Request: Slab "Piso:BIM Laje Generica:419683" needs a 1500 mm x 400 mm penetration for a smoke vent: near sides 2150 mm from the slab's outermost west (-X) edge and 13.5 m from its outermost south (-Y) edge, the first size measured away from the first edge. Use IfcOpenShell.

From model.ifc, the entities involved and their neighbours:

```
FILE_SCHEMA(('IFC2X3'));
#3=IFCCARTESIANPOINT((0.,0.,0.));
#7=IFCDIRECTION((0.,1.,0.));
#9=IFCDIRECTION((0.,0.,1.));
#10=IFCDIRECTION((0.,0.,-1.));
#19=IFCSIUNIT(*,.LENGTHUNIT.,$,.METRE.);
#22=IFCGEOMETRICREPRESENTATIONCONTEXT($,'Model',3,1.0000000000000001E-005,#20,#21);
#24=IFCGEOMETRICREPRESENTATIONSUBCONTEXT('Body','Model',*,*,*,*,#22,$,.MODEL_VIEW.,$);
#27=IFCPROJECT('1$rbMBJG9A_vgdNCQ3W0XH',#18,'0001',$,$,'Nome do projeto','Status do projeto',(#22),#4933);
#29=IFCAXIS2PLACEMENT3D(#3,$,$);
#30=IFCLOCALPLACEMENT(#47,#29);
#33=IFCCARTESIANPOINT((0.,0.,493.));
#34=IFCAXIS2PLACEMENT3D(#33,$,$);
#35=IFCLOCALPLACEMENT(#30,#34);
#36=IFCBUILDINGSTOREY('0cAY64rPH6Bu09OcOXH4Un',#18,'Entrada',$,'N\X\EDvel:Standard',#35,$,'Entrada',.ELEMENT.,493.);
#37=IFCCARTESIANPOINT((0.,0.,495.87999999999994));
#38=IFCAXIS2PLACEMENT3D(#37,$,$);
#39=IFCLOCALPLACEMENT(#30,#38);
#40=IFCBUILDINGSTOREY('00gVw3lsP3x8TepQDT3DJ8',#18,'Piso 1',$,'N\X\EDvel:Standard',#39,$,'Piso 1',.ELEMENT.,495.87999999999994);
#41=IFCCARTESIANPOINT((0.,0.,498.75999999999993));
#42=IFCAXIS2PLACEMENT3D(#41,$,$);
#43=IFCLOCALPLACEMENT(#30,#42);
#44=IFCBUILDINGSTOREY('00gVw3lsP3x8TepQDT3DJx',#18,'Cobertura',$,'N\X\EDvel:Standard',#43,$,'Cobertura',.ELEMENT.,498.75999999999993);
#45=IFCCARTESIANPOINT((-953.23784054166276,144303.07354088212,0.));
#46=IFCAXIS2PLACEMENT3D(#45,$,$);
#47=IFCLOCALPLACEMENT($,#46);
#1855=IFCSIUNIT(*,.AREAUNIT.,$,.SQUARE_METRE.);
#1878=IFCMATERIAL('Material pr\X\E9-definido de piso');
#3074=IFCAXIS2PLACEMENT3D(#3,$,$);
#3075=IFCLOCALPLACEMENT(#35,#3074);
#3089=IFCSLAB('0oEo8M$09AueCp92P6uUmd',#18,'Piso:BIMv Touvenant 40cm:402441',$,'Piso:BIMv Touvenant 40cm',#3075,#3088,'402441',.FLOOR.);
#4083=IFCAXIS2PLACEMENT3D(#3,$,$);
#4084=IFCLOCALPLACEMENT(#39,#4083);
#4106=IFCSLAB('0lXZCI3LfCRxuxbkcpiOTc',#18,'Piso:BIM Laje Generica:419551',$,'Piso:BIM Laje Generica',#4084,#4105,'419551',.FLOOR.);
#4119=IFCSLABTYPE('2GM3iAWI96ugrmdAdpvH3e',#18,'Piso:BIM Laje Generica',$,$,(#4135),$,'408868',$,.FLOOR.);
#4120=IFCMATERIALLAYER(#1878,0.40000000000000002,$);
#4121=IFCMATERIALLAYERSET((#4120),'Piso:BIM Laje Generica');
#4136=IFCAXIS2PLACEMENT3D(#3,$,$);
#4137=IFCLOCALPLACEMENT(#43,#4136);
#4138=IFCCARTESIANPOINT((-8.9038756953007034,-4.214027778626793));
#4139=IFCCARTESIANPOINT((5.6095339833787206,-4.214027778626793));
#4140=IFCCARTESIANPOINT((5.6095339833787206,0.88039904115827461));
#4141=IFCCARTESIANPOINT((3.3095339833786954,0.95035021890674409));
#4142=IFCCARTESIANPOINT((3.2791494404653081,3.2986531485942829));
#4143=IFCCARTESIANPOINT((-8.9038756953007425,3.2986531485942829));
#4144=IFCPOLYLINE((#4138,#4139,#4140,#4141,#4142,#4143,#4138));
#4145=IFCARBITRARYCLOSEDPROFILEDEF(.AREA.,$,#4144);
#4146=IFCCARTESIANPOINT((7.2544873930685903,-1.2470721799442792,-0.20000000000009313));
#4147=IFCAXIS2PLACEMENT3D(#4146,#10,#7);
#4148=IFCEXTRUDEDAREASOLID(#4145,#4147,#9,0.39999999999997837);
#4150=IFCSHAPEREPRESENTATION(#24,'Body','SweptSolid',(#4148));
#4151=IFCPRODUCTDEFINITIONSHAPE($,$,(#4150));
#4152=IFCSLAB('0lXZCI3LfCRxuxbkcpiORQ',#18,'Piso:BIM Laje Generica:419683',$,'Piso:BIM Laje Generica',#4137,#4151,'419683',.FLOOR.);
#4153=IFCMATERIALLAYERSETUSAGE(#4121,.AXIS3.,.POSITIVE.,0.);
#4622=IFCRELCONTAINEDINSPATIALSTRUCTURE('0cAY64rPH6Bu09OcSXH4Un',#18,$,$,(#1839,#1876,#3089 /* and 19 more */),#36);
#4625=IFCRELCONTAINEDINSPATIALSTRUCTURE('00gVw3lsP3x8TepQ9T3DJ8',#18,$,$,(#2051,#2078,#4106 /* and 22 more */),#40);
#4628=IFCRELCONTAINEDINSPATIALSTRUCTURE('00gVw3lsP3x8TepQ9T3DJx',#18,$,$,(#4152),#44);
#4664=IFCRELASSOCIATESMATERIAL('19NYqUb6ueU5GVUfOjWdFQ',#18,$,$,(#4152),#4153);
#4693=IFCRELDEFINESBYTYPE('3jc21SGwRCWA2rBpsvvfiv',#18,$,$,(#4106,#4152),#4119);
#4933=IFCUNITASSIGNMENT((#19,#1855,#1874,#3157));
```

```python
import numpy as np
import ifcopenshell
import ifcopenshell.api.feature
import ifcopenshell.api.geometry
import ifcopenshell.api.root
import ifcopenshell.geom
import ifcopenshell.util.placement
import ifcopenshell.util.representation
import ifcopenshell.util.shape
import ifcopenshell.util.unit

model = ifcopenshell.open("model.ifc")
unit_scale = ifcopenshell.util.unit.calculate_unit_scale(model)
settings = ifcopenshell.geom.settings()


def volume(element):
    """Net volume in cubic metres, openings subtracted."""
    shape = ifcopenshell.geom.create_shape(settings, element)
    return ifcopenshell.util.shape.get_volume(shape.geometry)


slab = model.by_id(4152)
before = volume(slab)

# Extent in the slab's own axes, in metres. The edges named are its -X and -Y sides.
slab_shape = ifcopenshell.geom.create_shape(settings, slab)
vertices = ifcopenshell.util.shape.get_vertices(slab_shape.geometry)
x_min, y_min, bottom = vertices.min(axis=0)
top = vertices[:, 2].max()

opening = ifcopenshell.api.root.create_entity(model, ifc_class="IfcOpeningElement", name="Smoke vent opening")
context = ifcopenshell.util.representation.get_context(model, "Model", "Body", "MODEL_VIEW")
width, depth = 1.5, 0.4
outline = [(0.0, 0.0), (width, 0.0), (width, depth), (0.0, depth), (0.0, 0.0)]
# Overshoot both faces by 50 mm so the cut is clean.
shape = ifcopenshell.api.geometry.add_slab_representation(
    model, context=context, depth=top - bottom + 0.1, polyline=outline
)
ifcopenshell.api.geometry.assign_representation(model, product=opening, representation=shape)

matrix = ifcopenshell.util.placement.get_local_placement(slab.ObjectPlacement)
matrix[:, 3] = matrix @ np.append(np.array([x_min + 2.15, y_min + 13.5, bottom - 0.05]) / unit_scale, 1.0)
ifcopenshell.api.geometry.edit_object_placement(model, product=opening, matrix=matrix, is_si=False)
ifcopenshell.api.feature.add_feature(model, feature=opening, element=slab)

after = volume(slab)

print(f"slab volume {before:.3f} -> {after:.3f} m3")

model.write("model_rev.ifc")
```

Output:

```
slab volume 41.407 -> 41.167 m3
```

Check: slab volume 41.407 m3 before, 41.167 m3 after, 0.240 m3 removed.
